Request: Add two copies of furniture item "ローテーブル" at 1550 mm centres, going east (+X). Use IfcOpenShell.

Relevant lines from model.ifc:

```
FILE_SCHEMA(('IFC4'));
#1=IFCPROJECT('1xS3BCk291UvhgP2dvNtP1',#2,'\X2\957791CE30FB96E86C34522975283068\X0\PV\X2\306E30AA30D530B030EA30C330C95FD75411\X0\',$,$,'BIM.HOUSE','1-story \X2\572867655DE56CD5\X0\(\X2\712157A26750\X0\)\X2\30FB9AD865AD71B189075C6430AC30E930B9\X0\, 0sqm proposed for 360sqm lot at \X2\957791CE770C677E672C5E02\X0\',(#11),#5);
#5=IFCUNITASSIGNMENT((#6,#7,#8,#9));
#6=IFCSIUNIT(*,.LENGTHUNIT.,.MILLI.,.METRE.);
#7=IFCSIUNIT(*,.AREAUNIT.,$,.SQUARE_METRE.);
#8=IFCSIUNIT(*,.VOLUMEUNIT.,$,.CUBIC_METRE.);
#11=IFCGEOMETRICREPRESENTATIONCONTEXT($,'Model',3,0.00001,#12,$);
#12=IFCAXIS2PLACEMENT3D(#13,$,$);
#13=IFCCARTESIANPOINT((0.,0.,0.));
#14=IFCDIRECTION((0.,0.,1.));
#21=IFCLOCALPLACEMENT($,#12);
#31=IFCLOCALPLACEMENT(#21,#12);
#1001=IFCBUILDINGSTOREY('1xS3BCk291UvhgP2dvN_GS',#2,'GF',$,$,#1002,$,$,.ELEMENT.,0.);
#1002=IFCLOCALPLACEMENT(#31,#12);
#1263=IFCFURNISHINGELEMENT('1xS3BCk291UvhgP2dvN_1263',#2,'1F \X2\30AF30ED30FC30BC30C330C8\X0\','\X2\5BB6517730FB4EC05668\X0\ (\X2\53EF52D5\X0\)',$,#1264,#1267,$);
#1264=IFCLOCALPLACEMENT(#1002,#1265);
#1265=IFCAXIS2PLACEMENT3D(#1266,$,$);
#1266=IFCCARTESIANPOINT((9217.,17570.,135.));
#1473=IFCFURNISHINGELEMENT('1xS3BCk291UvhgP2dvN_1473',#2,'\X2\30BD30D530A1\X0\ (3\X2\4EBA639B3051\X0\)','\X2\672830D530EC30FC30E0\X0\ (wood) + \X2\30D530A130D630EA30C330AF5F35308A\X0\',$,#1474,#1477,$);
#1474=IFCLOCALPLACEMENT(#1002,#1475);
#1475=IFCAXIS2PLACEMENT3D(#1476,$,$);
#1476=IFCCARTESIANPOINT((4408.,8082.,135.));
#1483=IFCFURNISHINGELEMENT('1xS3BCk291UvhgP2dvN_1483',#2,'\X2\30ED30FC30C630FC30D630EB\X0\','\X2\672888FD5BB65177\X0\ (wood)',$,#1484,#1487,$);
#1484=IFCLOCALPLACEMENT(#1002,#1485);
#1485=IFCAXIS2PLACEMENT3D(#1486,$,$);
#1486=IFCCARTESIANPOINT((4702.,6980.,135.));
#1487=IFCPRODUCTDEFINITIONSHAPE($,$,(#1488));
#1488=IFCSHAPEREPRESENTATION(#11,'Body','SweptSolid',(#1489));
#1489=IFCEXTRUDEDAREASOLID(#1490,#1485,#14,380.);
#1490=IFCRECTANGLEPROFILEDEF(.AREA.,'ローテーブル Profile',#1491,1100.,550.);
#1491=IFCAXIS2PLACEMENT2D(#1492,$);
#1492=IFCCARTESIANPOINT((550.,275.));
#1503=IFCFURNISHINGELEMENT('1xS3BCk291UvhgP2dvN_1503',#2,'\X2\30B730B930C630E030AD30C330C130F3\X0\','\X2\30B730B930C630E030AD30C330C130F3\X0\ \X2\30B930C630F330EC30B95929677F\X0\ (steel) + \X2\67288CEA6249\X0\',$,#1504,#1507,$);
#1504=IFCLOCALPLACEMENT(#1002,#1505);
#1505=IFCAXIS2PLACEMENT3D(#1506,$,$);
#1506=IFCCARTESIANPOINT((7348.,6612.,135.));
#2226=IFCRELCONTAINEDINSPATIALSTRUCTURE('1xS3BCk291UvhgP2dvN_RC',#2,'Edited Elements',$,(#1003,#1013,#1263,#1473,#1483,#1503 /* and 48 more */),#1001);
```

```python
import numpy as np
import ifcopenshell
import ifcopenshell.api.geometry
import ifcopenshell.api.root
import ifcopenshell.util.element
import ifcopenshell.util.placement

model = ifcopenshell.open("model.ifc")


def reuse_history(source, copy):
    """copy_class also copies each property set's owner history, people and application; keep the originals."""
    for rel in copy.IsDefinedBy:
        if rel.is_a("IfcRelDefinesByProperties") and (history := rel.RelatingPropertyDefinition.OwnerHistory):
            rel.RelatingPropertyDefinition.OwnerHistory = source.OwnerHistory
            ifcopenshell.util.element.remove_deep2(model, history)


source = model.by_guid("1xS3BCk291UvhgP2dvN_1483")
base = ifcopenshell.util.placement.get_local_placement(source.ObjectPlacement)
step = np.array([1.0, 0.0, 0.0]) * 1550.0

for i in range(1, 3):
    copy = ifcopenshell.api.root.copy_class(model, product=source)
    copy.Representation = ifcopenshell.util.element.copy_deep(
        model, source.Representation, exclude=["IfcGeometricRepresentationContext", "IfcRepresentationMap"]
    )
    reuse_history(source, copy)
    matrix = base.copy()
    matrix[:3, 3] += i * step
    print("added at", matrix[:3, 3].round(3) + 0.0)
    ifcopenshell.api.geometry.edit_object_placement(model, product=copy, matrix=matrix, is_si=False)

model.write("model-out.ifc")
```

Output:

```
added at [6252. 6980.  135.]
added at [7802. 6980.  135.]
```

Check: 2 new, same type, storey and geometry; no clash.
